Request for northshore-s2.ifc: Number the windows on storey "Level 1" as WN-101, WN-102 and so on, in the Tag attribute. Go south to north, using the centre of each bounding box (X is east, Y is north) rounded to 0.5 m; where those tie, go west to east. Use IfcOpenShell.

First a look at what the model holds.

```python
import ifcopenshell
import ifcopenshell.util.element
import ifcopenshell.util.placement

model = ifcopenshell.open("northshore-s2.ifc")
print(model.schema)
storey = next(s for s in model.by_type("IfcBuildingStorey") if s.Name == "Level 1")
windows = [e for e in ifcopenshell.util.element.get_decomposition(storey) if e.is_a("IfcWindow")]
for e in sorted(windows, key=lambda e: e.id()):
    origin = ifcopenshell.util.placement.get_local_placement(e.ObjectPlacement)[:3, 3]
    print(e.id(), e.Tag, e.Name, origin.round(2) + 0.0, sep=" | ")
```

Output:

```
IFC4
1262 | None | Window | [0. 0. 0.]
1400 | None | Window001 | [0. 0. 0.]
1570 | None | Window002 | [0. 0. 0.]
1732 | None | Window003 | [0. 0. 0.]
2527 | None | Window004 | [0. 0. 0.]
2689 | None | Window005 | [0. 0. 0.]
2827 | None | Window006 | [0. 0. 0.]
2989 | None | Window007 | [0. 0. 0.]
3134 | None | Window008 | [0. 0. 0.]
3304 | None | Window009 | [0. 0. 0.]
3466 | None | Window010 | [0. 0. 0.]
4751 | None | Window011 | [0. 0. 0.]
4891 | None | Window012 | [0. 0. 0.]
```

```python
import ifcopenshell
import ifcopenshell.geom
import ifcopenshell.util.element
import ifcopenshell.util.shape

model = ifcopenshell.open("northshore-s2.ifc")
settings = ifcopenshell.geom.settings()
settings.set("use-world-coords", True)


def centre(element):
    shape = ifcopenshell.geom.create_shape(settings, element)
    return ifcopenshell.util.shape.get_bbox_centroid(shape.geometry)


storey = next(s for s in model.by_type("IfcBuildingStorey") if s.Name == "Level 1")
windows = [e for e in ifcopenshell.util.element.get_decomposition(storey) if e.is_a("IfcWindow")]

# Insertion points can sit at a corner or the storey origin, so sort by the geometry (in metres).
centres = {e: centre(e) for e in windows}
windows.sort(key=lambda e: (round(centres[e][1] / 0.5), centres[e][0]))

for i, e in enumerate(windows, start=1):
    number = f"WN-1{i:02d}"
    e.Tag = number
    print(e.id(), number)

model.write("northshore-s2-out.ifc")
```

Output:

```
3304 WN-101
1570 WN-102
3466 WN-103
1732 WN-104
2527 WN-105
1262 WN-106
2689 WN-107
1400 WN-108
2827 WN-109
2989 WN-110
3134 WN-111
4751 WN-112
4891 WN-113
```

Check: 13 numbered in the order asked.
